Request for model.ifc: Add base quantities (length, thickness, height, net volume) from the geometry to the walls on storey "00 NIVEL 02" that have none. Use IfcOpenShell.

First a look at what the model holds.

```python
import ifcopenshell
import ifcopenshell.util.element
import ifcopenshell.util.unit

model = ifcopenshell.open("model.ifc")
print(model.schema)
for unit_type in ("LENGTHUNIT", "AREAUNIT", "VOLUMEUNIT"):
    print(unit_type, ifcopenshell.util.unit.calculate_unit_scale(model, unit_type))
storey = next(s for s in model.by_type("IfcBuildingStorey") if s.Name == "00 NIVEL 02")
walls = [e for e in ifcopenshell.util.element.get_decomposition(storey) if e.is_a("IfcWall")]
for e in sorted(walls, key=lambda e: e.id()):
    print(e.id(), e.is_a(), e.Name, list(ifcopenshell.util.element.get_psets(e, qtos_only=True)), sep=" | ")
```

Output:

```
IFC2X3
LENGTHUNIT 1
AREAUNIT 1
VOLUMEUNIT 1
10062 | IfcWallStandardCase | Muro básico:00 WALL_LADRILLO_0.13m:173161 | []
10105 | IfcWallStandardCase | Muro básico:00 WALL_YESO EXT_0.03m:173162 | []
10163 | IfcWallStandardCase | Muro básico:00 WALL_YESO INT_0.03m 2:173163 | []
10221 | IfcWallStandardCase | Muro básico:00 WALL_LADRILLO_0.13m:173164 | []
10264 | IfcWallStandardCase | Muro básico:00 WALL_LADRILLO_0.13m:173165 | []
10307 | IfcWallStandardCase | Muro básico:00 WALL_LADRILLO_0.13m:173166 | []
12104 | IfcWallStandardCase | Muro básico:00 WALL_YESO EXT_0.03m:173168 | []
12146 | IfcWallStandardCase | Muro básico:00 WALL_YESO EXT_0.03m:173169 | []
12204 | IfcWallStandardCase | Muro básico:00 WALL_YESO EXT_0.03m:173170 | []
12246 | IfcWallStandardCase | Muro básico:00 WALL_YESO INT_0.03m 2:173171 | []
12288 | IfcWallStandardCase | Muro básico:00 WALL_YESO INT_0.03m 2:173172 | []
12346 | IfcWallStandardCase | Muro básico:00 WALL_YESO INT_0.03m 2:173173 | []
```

```python
import ifcopenshell
import ifcopenshell.api.pset
import ifcopenshell.geom
import ifcopenshell.util.element
import ifcopenshell.util.shape
import ifcopenshell.util.unit

model = ifcopenshell.open("model.ifc")
unit_scale = ifcopenshell.util.unit.calculate_unit_scale(model)
volume_scale = ifcopenshell.util.unit.calculate_unit_scale(model, "VOLUMEUNIT")
settings = ifcopenshell.geom.settings()

storey = next(s for s in model.by_type("IfcBuildingStorey") if s.Name == "00 NIVEL 02")
walls = [e for e in ifcopenshell.util.element.get_decomposition(storey) if e.is_a("IfcWall")]

for e in sorted(walls, key=lambda e: e.id()):
    if ifcopenshell.util.element.get_psets(e, qtos_only=True, should_inherit=False):
        continue
    # Geometry comes back in metres, in the element's own axes.
    shape = ifcopenshell.geom.create_shape(settings, e)
    values = {
        "Length": ifcopenshell.util.shape.get_x(shape.geometry) / unit_scale,
        "Width": ifcopenshell.util.shape.get_y(shape.geometry) / unit_scale,
        "Height": ifcopenshell.util.shape.get_z(shape.geometry) / unit_scale,
        "NetVolume": ifcopenshell.util.shape.get_volume(shape.geometry) / volume_scale,
    }
    qto = ifcopenshell.api.pset.add_qto(model, product=e, name="BaseQuantities")
    ifcopenshell.api.pset.edit_qto(model, qto=qto, properties=values)
    print(e.id(), {k: round(v, 3) for k, v in values.items()})

model.write("model_rev.ifc")
```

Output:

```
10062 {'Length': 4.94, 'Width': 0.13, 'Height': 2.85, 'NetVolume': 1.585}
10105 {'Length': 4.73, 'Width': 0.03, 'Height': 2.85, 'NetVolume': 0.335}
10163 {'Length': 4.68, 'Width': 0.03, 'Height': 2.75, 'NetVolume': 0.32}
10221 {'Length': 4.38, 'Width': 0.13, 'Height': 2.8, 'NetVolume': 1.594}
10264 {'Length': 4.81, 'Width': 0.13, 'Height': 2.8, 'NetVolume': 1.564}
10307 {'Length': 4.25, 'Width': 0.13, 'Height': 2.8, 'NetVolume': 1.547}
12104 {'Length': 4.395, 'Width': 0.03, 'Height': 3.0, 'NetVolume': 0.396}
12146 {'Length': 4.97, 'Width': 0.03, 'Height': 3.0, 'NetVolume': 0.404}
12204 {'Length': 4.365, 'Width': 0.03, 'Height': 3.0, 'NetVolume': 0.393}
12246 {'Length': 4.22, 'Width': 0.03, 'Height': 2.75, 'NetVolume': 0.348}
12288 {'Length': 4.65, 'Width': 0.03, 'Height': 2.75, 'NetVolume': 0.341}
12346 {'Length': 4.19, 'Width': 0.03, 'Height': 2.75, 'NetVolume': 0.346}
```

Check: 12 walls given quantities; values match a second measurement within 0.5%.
